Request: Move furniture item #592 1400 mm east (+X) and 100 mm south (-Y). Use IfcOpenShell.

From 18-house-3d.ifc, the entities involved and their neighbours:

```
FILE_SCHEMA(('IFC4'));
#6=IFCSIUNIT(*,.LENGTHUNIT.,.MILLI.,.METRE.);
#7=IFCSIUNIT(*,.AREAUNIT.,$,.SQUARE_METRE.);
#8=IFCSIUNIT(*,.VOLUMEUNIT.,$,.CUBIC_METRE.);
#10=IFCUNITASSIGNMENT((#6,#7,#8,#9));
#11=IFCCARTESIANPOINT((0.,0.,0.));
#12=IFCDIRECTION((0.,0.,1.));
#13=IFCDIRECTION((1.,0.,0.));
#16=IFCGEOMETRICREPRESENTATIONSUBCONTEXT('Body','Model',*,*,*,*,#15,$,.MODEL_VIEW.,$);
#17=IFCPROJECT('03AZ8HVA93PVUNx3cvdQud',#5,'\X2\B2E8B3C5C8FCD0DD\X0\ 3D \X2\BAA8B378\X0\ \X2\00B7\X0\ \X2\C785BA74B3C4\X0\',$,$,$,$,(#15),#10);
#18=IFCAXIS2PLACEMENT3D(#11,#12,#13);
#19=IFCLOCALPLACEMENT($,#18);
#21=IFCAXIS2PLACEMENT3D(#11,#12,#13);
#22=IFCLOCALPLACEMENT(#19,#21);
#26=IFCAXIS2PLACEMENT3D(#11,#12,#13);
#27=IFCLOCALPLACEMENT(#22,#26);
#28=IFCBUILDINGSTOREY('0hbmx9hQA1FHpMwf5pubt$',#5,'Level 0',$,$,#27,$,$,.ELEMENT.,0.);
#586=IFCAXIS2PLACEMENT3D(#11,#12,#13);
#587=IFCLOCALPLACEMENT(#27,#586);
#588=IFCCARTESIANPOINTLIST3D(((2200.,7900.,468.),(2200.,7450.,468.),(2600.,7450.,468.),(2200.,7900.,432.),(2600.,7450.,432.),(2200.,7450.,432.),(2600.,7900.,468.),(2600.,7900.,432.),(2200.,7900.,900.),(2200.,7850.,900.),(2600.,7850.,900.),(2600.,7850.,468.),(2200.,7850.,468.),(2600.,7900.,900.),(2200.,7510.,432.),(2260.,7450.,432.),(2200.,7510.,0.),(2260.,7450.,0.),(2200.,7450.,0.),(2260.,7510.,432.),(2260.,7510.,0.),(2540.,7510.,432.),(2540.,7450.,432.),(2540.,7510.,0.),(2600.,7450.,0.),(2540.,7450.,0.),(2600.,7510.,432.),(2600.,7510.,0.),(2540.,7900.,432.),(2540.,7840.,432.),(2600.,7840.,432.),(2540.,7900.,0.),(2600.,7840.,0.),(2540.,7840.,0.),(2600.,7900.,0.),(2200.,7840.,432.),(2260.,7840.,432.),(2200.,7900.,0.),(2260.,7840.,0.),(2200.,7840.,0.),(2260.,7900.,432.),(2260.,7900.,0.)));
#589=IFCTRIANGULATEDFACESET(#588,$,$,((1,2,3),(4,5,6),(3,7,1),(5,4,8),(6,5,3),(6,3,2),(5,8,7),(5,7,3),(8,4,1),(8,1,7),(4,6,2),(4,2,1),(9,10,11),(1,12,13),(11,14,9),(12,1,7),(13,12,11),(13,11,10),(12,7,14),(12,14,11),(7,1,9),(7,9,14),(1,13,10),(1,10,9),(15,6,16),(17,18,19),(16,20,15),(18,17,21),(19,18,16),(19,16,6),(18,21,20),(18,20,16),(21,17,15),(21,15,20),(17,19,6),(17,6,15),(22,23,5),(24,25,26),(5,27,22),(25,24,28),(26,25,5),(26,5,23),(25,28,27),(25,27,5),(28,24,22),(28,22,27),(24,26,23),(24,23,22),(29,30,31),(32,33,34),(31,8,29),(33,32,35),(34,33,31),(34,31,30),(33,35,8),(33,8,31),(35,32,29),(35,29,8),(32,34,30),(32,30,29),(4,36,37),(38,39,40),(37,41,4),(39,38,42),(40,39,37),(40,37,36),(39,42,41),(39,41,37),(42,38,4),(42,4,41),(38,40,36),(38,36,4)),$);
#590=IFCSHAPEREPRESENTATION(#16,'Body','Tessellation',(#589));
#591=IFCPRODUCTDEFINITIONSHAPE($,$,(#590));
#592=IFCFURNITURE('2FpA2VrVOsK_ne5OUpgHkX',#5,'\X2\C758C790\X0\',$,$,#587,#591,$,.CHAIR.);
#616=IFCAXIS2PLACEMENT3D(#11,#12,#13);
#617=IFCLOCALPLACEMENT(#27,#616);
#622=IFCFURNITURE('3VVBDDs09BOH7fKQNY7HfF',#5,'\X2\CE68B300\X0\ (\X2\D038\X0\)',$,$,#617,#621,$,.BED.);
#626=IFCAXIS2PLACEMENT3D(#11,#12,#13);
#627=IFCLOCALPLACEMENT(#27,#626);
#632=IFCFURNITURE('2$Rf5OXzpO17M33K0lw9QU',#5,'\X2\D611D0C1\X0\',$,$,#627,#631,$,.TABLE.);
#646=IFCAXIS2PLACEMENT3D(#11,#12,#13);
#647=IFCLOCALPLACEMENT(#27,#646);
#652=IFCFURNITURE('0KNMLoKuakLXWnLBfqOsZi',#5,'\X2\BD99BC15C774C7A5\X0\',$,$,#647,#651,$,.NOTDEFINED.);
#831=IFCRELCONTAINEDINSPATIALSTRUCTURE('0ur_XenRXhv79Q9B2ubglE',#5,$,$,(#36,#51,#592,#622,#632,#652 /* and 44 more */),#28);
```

```python
import ifcopenshell
import ifcopenshell.api.geometry
import ifcopenshell.util.placement

model = ifcopenshell.open("18-house-3d.ifc")

item = model.by_guid("2FpA2VrVOsK_ne5OUpgHkX")
matrix = ifcopenshell.util.placement.get_local_placement(item.ObjectPlacement)
matrix[0, 3] += 1400.0
matrix[1, 3] -= 100.0
ifcopenshell.api.geometry.edit_object_placement(model, product=item, matrix=matrix, is_si=False)

print(ifcopenshell.util.placement.get_local_placement(item.ObjectPlacement).round(3) + 0.0)

model.write("18-house-3d_v2.ifc")
```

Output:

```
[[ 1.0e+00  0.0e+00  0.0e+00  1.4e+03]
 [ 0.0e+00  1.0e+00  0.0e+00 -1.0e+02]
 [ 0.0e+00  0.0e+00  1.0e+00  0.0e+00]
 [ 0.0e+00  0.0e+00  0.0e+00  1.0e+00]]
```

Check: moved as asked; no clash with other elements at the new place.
